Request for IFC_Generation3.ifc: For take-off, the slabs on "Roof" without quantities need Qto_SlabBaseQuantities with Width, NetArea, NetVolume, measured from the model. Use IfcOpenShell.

First a look at what the model holds.

```python
import ifcopenshell
import ifcopenshell.util.element
import ifcopenshell.util.unit

model = ifcopenshell.open("IFC_Generation3.ifc")
print(model.schema)
for unit_type in ("LENGTHUNIT", "AREAUNIT", "VOLUMEUNIT"):
    print(unit_type, ifcopenshell.util.unit.calculate_unit_scale(model, unit_type))
storey = next(s for s in model.by_type("IfcBuildingStorey") if s.Name == "Roof")
slabs = [e for e in ifcopenshell.util.element.get_decomposition(storey) if e.is_a("IfcSlab")]
for e in sorted(slabs, key=lambda e: e.id()):
    print(e.id(), e.is_a(), e.Name, list(ifcopenshell.util.element.get_psets(e, qtos_only=True)), sep=" | ")
```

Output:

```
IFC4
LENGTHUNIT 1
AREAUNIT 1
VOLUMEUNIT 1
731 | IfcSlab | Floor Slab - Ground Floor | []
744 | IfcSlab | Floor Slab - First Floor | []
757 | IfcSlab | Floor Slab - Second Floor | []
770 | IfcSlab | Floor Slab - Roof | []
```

```python
import ifcopenshell
import ifcopenshell.api.pset
import ifcopenshell.geom
import ifcopenshell.util.element
import ifcopenshell.util.shape
import ifcopenshell.util.unit

model = ifcopenshell.open("IFC_Generation3.ifc")
unit_scale = ifcopenshell.util.unit.calculate_unit_scale(model)
area_scale = ifcopenshell.util.unit.calculate_unit_scale(model, "AREAUNIT")
volume_scale = ifcopenshell.util.unit.calculate_unit_scale(model, "VOLUMEUNIT")
settings = ifcopenshell.geom.settings()

storey = next(s for s in model.by_type("IfcBuildingStorey") if s.Name == "Roof")
slabs = [e for e in ifcopenshell.util.element.get_decomposition(storey) if e.is_a("IfcSlab")]

for e in sorted(slabs, key=lambda e: e.id()):
    if ifcopenshell.util.element.get_psets(e, qtos_only=True, should_inherit=False):
        continue
    # Geometry comes back in metres, in the element's own axes.
    shape = ifcopenshell.geom.create_shape(settings, e)
    values = {
        "Width": ifcopenshell.util.shape.get_z(shape.geometry) / unit_scale,
        "NetArea": ifcopenshell.util.shape.get_footprint_area(shape.geometry) / area_scale,
        "NetVolume": ifcopenshell.util.shape.get_volume(shape.geometry) / volume_scale,
    }
    qto = ifcopenshell.api.pset.add_qto(model, product=e, name="Qto_SlabBaseQuantities")
    ifcopenshell.api.pset.edit_qto(model, qto=qto, properties=values)
    print(e.id(), {k: round(v, 3) for k, v in values.items()})

model.write("IFC_Generation3-out.ifc")
```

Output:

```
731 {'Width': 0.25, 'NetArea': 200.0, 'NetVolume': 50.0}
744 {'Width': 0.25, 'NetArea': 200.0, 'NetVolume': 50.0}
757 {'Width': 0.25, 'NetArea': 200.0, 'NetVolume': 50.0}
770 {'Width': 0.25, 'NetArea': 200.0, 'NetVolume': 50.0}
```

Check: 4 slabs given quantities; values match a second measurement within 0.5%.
